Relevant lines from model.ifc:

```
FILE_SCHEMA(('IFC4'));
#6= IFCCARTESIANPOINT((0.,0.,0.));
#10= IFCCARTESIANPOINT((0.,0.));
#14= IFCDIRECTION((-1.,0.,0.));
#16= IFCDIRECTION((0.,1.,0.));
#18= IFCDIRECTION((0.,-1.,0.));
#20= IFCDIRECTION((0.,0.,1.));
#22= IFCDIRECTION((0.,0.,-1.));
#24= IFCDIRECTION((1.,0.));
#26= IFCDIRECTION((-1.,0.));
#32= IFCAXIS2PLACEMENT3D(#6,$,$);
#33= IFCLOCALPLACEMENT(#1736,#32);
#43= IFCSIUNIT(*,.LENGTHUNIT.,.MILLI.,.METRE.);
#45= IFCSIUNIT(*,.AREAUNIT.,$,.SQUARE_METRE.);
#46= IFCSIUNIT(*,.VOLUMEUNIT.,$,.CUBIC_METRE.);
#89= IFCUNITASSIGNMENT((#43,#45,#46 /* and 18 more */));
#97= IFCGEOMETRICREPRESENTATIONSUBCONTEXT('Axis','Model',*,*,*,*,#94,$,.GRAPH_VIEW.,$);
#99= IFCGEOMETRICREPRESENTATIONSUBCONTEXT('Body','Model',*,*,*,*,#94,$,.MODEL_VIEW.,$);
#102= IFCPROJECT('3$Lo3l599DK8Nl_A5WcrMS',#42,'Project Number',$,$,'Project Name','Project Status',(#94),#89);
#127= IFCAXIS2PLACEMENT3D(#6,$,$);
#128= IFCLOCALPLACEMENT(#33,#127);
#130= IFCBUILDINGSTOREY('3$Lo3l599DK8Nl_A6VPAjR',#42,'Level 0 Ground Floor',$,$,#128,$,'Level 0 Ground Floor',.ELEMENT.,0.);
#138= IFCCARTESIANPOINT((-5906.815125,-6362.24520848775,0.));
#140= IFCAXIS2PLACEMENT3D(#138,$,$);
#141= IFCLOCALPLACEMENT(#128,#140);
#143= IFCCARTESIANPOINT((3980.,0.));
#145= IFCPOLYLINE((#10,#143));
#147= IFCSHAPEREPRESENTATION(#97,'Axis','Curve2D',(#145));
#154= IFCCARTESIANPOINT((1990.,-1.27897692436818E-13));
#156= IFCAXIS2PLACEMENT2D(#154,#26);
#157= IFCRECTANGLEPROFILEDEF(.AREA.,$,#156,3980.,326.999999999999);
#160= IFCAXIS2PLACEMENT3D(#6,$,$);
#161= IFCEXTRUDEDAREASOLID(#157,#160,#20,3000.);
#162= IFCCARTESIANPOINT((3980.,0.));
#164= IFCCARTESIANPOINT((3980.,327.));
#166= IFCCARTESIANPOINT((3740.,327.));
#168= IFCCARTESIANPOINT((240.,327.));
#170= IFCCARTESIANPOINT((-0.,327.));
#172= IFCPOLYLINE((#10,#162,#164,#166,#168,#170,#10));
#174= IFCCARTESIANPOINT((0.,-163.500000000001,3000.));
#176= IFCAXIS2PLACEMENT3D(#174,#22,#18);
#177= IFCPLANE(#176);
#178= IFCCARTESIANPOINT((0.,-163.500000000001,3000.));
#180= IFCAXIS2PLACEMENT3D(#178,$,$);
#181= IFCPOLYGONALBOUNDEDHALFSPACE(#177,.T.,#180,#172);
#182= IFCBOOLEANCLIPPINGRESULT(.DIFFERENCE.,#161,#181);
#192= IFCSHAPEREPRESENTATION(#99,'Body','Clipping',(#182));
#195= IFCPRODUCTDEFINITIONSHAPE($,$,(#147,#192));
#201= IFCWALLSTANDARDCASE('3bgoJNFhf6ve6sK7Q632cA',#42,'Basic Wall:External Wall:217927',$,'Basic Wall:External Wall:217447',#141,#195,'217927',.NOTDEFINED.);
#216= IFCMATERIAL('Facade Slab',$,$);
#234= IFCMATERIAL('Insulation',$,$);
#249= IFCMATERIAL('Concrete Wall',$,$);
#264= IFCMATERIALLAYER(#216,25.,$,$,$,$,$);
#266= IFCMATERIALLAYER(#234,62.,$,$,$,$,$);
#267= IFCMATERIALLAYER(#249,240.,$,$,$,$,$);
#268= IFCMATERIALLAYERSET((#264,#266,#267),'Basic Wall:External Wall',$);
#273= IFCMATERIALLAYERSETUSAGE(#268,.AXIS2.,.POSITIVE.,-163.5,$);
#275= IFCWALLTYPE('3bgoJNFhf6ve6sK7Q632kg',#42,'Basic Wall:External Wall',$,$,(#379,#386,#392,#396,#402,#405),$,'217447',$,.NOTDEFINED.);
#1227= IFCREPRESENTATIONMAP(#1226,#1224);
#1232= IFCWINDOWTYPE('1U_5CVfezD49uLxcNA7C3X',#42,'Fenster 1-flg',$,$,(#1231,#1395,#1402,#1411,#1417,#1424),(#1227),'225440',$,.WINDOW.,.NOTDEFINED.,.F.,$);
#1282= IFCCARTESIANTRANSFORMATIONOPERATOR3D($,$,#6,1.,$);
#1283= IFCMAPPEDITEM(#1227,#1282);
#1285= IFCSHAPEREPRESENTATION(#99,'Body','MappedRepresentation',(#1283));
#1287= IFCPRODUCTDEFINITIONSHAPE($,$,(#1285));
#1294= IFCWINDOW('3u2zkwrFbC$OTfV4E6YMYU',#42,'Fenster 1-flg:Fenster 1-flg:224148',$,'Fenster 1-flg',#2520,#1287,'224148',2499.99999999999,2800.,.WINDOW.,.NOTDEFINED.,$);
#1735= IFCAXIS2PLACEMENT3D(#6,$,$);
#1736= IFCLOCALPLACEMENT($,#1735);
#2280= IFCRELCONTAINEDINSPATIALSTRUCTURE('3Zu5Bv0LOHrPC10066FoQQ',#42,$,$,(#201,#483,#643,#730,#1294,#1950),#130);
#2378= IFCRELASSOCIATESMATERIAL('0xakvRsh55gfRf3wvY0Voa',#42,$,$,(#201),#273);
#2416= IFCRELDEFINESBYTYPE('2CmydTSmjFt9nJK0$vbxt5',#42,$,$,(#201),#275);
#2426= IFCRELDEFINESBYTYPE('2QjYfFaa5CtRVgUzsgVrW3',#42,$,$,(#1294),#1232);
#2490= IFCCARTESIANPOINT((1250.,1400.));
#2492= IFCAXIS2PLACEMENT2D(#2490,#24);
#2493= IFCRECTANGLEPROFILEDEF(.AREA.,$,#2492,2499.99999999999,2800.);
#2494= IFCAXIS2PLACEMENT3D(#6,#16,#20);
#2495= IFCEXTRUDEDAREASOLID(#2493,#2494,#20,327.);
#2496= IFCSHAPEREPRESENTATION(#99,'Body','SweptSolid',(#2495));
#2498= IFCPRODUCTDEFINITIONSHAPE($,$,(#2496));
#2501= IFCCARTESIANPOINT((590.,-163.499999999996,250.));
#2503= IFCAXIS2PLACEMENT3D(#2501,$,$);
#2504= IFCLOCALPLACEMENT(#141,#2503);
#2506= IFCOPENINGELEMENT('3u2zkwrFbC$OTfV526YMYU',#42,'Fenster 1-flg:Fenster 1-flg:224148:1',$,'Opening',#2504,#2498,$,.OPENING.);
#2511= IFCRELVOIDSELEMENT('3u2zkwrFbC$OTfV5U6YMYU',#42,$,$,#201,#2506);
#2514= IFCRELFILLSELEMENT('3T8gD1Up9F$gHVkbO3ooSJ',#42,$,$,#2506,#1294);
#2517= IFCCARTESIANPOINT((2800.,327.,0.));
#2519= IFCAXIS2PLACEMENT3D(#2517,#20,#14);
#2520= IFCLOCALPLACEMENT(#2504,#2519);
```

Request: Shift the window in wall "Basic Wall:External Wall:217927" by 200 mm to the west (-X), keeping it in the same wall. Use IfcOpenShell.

```python
import ifcopenshell
import ifcopenshell.api.geometry
import ifcopenshell.util.placement
import ifcopenshell.util.unit

model = ifcopenshell.open("model.ifc")
unit_scale = ifcopenshell.util.unit.calculate_unit_scale(model)

window = model.by_guid("3u2zkwrFbC$OTfV4E6YMYU")
opening = window.FillsVoids[0].RelatingOpeningElement
wall = opening.VoidsElements[0].RelatingBuildingElement

wall_matrix = ifcopenshell.util.placement.get_local_placement(wall.ObjectPlacement)
shift = wall_matrix[:3, 0] * -0.2 / unit_scale
before = ifcopenshell.util.placement.get_local_placement(window.ObjectPlacement)[:3, 3].copy()

# The window is placed relative to its opening, so it follows when the opening moves.
matrix = ifcopenshell.util.placement.get_local_placement(opening.ObjectPlacement)
matrix[:3, 3] += shift
ifcopenshell.api.geometry.edit_object_placement(
    model, product=opening, matrix=matrix, is_si=False, should_transform_children=True
)

after = ifcopenshell.util.placement.get_local_placement(window.ObjectPlacement)[:3, 3]
print("window moved by", (after - before).round(3) + 0.0)

model.write("model-out.ifc")
```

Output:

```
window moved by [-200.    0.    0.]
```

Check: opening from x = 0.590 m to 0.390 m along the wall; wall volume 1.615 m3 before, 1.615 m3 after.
